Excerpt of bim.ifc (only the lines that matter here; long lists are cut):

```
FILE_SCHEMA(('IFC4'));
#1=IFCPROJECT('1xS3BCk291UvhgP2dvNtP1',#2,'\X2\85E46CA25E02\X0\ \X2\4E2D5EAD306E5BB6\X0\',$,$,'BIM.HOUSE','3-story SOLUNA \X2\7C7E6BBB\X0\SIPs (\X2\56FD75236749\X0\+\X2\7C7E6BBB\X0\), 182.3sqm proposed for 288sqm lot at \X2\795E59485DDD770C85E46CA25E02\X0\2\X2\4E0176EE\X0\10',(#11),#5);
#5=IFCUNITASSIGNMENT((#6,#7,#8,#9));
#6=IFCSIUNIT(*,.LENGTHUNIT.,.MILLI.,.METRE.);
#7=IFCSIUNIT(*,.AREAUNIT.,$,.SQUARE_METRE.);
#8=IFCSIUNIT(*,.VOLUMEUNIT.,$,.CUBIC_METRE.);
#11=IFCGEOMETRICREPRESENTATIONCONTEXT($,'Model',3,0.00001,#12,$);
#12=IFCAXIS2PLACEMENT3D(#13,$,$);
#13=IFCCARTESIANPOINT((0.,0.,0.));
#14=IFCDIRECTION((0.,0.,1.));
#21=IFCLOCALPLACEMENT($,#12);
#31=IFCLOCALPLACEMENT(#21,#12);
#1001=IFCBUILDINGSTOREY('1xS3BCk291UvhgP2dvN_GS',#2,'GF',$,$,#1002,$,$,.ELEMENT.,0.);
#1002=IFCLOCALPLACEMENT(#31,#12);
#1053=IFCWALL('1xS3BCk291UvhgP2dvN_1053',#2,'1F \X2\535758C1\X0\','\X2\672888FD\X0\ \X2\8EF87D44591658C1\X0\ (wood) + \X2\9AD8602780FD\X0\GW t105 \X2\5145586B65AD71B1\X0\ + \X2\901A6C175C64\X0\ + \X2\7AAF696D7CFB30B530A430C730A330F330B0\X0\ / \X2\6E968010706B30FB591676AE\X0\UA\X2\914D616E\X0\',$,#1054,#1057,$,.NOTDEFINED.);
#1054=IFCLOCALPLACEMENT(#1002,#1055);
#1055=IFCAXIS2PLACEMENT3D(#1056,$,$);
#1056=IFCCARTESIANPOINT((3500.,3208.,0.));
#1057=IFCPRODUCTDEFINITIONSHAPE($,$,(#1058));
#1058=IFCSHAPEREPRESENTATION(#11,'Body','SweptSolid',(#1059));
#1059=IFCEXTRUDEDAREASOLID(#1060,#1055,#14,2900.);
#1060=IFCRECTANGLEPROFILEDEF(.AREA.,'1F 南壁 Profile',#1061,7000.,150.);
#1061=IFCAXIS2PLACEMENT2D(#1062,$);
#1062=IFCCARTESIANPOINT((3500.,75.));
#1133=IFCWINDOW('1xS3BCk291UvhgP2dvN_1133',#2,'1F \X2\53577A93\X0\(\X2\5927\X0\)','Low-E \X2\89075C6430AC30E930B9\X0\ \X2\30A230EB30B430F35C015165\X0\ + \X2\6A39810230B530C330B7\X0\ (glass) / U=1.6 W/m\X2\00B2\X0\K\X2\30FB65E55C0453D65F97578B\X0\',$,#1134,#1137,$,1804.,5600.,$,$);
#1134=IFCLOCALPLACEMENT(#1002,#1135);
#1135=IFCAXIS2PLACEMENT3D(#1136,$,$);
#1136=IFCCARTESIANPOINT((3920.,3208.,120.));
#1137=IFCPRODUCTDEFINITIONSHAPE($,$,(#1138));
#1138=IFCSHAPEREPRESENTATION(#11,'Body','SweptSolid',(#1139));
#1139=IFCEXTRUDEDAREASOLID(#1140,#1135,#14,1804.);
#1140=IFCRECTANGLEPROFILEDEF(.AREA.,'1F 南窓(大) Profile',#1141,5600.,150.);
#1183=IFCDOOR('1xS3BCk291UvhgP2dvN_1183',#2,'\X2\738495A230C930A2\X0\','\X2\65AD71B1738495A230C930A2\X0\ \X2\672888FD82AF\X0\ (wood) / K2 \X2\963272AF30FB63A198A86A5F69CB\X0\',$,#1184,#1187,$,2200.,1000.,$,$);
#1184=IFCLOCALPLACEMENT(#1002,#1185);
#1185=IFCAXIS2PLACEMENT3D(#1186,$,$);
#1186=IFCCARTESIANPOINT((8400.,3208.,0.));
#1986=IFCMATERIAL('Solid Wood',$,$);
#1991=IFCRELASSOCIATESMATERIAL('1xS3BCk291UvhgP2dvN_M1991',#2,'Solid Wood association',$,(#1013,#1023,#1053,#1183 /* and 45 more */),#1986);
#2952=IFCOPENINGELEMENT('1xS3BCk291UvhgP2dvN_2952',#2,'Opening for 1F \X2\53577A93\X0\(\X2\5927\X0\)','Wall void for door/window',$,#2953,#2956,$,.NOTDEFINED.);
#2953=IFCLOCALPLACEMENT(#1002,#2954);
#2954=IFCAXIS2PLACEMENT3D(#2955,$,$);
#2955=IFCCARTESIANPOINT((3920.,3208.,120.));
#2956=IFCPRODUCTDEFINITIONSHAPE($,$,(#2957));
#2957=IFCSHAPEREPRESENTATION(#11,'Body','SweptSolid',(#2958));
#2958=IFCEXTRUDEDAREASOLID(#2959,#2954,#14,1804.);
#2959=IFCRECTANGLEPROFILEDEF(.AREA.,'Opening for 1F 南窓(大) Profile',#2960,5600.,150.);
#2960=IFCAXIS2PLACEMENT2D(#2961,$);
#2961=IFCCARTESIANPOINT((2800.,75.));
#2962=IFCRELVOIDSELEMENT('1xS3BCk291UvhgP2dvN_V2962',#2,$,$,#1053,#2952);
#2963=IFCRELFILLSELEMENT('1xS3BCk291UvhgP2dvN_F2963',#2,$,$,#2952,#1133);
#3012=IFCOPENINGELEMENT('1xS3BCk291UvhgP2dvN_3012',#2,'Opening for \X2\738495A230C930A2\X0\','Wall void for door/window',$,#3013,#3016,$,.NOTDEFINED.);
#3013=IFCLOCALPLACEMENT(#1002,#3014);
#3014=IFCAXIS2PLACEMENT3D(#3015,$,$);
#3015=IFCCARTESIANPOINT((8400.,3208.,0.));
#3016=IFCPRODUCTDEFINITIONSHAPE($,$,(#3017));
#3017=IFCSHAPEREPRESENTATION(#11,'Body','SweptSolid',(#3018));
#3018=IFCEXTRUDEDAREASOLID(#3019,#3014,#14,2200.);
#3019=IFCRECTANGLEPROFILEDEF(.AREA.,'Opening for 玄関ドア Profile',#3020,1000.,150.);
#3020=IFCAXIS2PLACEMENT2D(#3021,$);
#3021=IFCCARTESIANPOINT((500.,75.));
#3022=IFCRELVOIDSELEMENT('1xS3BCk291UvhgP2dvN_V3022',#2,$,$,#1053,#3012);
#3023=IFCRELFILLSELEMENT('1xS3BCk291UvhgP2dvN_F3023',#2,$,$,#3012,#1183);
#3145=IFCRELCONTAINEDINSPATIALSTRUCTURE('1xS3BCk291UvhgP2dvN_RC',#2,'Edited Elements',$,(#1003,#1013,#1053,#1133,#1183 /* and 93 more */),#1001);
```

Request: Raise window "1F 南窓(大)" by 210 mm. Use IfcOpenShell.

```python
import numpy as np
import ifcopenshell
import ifcopenshell.api.geometry
import ifcopenshell.util.placement
import ifcopenshell.util.unit

model = ifcopenshell.open("bim.ifc")
unit_scale = ifcopenshell.util.unit.calculate_unit_scale(model)

window = model.by_id(1133)
opening = window.FillsVoids[0].RelatingOpeningElement
dz = 210.0

shift = np.array([0.0, 0.0, dz])
# The window is not placed relative to its opening, so move both.
for product in (opening, window):
    matrix = ifcopenshell.util.placement.get_local_placement(product.ObjectPlacement)
    matrix[:3, 3] += shift
    ifcopenshell.api.geometry.edit_object_placement(model, product=product, matrix=matrix, is_si=False)

print(f"moved by {dz * unit_scale:+.3f} m")

model.write("bim_v2.ifc")
```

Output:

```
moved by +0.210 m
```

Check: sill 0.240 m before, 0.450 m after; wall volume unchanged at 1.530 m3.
